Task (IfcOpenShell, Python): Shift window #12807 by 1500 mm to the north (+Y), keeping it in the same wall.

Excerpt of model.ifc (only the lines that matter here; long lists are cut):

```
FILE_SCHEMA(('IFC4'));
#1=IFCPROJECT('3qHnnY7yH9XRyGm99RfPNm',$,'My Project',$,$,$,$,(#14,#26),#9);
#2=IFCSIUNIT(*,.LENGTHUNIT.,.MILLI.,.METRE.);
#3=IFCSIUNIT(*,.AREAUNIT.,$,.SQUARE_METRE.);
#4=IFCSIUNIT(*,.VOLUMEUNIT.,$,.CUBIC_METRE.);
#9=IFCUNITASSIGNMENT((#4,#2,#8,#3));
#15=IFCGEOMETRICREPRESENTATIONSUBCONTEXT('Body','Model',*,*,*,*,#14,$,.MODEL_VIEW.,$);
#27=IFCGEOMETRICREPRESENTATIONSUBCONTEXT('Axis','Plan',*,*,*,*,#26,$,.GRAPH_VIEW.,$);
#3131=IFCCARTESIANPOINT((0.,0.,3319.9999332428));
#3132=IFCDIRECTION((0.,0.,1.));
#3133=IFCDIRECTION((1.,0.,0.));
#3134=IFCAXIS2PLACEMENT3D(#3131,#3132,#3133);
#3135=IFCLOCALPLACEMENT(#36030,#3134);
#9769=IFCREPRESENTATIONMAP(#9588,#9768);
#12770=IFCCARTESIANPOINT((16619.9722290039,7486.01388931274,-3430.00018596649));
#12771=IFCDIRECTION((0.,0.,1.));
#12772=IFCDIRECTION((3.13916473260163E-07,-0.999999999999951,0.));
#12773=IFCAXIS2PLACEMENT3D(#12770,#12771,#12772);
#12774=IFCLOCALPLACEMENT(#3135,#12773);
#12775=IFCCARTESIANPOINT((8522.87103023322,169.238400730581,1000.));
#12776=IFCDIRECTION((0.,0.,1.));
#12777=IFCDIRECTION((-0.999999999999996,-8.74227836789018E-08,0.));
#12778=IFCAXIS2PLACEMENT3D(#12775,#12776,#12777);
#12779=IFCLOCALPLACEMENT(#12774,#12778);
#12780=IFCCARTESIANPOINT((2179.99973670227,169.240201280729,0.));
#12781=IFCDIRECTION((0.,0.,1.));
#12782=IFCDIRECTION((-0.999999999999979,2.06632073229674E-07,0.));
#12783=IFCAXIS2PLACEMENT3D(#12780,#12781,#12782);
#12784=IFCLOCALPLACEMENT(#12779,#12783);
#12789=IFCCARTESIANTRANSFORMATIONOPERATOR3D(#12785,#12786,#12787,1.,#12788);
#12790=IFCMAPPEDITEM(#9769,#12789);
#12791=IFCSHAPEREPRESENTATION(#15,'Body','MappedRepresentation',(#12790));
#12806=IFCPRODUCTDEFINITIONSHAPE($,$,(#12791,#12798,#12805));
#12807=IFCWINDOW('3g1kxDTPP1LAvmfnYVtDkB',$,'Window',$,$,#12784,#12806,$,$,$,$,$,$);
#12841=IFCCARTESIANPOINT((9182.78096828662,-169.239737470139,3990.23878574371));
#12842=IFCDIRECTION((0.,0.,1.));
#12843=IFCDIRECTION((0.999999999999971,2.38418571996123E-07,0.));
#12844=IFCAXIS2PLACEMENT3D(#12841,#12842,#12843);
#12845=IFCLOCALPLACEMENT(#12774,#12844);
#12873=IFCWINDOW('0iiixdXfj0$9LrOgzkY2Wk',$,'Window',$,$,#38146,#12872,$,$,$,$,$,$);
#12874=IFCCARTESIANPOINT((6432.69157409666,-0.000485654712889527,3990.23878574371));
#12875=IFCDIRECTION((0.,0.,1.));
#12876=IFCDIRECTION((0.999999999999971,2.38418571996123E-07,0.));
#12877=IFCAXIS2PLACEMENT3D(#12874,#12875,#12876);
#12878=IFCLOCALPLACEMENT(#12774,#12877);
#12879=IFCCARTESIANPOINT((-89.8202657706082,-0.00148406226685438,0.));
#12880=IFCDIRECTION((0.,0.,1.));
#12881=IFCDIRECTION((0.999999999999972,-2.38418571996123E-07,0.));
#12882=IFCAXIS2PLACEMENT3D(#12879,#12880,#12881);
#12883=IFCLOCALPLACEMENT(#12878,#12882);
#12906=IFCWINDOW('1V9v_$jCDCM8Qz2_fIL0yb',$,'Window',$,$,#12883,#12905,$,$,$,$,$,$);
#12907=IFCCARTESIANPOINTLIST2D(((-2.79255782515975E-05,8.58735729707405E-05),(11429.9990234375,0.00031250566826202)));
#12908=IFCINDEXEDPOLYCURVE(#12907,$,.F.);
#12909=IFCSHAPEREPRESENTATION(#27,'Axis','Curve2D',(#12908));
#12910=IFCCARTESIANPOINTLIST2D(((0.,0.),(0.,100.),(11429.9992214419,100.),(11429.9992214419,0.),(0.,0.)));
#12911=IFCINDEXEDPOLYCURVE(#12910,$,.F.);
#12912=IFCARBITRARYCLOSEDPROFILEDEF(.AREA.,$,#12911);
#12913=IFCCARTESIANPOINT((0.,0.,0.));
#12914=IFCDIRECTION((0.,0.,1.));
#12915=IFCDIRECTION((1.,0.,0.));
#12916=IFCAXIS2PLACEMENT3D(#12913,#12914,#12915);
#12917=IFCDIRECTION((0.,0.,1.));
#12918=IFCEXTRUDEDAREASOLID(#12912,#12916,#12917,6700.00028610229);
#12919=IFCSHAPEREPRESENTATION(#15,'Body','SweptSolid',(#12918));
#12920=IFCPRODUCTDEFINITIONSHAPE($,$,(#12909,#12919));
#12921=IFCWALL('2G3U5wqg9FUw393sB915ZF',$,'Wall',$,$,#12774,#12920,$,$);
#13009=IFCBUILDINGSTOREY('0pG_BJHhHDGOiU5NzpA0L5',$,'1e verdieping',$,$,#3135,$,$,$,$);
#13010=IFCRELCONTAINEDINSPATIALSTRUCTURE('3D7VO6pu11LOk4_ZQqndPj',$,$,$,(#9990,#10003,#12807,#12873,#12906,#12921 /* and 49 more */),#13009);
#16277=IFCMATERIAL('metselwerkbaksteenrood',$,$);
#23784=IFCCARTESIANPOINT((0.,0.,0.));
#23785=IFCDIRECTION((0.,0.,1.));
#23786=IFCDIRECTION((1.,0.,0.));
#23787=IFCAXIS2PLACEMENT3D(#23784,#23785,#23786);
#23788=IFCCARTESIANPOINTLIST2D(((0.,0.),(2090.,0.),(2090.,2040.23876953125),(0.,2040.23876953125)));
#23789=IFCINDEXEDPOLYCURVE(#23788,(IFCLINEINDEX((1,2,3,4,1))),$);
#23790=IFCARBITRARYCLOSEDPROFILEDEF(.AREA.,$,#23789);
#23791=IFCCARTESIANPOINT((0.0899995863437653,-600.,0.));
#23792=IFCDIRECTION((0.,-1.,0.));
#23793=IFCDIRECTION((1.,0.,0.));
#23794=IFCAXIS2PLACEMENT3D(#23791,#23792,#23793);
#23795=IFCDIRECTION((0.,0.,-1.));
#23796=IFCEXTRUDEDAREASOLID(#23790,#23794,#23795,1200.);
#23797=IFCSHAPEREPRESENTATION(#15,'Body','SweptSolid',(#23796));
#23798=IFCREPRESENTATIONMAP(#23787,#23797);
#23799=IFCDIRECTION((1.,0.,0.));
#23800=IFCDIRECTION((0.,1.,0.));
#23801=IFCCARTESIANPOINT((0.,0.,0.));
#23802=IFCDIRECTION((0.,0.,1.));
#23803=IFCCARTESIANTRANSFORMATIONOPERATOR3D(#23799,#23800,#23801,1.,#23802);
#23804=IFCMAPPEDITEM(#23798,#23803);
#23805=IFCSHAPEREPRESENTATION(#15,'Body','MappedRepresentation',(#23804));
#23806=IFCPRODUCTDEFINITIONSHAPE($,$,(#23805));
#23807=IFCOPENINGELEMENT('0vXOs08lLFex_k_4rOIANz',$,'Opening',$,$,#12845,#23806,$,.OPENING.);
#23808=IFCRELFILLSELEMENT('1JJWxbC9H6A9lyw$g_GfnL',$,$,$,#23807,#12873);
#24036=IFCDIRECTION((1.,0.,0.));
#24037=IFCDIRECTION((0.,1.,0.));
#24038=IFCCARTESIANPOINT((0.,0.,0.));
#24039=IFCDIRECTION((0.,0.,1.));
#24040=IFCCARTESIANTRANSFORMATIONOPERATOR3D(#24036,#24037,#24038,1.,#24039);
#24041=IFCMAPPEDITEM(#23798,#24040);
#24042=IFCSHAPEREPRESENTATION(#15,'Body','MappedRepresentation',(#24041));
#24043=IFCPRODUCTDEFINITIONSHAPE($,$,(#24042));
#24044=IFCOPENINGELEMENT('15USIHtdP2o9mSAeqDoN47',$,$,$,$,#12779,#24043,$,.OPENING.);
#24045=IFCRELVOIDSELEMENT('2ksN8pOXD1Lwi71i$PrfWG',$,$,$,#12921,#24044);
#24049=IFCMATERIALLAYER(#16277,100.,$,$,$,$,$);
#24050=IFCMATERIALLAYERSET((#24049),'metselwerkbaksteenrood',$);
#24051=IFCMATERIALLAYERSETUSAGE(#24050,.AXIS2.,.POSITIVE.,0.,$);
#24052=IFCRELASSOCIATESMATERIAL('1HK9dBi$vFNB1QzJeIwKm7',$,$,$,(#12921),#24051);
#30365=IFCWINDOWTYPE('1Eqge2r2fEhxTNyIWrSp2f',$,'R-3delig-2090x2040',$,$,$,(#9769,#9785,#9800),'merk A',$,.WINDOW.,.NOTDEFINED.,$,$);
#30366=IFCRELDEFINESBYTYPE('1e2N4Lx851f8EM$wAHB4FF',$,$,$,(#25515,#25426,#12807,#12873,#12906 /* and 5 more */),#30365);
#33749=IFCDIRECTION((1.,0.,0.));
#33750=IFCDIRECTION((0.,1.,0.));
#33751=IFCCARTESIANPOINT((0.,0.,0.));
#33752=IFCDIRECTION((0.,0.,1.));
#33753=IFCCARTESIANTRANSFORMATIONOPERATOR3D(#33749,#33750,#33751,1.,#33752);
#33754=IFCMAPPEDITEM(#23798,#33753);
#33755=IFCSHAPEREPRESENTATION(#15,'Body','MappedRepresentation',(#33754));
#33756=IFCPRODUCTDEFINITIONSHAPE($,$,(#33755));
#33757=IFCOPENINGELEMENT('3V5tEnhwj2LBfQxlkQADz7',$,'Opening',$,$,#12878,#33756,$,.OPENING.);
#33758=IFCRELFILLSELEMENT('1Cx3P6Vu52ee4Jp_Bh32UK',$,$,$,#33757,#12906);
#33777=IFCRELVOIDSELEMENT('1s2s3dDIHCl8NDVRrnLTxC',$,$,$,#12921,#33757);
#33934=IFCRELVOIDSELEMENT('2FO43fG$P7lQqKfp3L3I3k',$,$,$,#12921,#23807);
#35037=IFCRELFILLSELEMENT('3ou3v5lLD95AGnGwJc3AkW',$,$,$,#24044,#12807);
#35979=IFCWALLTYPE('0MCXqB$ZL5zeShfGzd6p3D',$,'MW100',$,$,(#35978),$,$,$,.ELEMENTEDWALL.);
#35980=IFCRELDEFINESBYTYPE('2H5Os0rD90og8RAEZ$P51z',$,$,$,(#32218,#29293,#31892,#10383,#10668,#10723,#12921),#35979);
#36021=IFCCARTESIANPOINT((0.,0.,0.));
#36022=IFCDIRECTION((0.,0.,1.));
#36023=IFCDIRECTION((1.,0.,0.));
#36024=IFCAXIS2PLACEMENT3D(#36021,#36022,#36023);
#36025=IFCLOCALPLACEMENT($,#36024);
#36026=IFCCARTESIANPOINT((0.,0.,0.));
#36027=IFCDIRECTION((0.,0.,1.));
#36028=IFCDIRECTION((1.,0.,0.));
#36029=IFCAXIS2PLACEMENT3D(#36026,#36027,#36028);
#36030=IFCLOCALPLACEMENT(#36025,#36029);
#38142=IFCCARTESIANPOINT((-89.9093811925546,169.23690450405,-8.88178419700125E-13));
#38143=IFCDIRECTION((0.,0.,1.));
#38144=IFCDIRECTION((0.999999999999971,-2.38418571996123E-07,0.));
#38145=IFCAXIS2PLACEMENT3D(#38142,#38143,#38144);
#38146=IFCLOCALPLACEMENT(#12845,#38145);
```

```python
import ifcopenshell
import ifcopenshell.api.geometry
import ifcopenshell.util.placement
import ifcopenshell.util.unit

model = ifcopenshell.open("model.ifc")
unit_scale = ifcopenshell.util.unit.calculate_unit_scale(model)

window = model.by_guid("3g1kxDTPP1LAvmfnYVtDkB")
opening = window.FillsVoids[0].RelatingOpeningElement
wall = opening.VoidsElements[0].RelatingBuildingElement

wall_matrix = ifcopenshell.util.placement.get_local_placement(wall.ObjectPlacement)
shift = wall_matrix[:3, 0] * -1.5 / unit_scale
before = ifcopenshell.util.placement.get_local_placement(window.ObjectPlacement)[:3, 3].copy()

# The window is placed relative to its opening, so it follows when the opening moves.
matrix = ifcopenshell.util.placement.get_local_placement(opening.ObjectPlacement)
matrix[:3, 3] += shift
ifcopenshell.api.geometry.edit_object_placement(
    model, product=opening, matrix=matrix, is_si=False, should_transform_children=True
)

after = ifcopenshell.util.placement.get_local_placement(window.ObjectPlacement)[:3, 3]
print("window moved by", (after - before).round(3) + 0.0)

model.write("model_v2.ifc")
```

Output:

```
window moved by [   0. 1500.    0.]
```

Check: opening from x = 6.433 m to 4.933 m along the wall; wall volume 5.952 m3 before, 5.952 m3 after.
